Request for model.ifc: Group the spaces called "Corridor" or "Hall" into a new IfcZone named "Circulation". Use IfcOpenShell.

First a look at what the model holds.

```python
import ifcopenshell

model = ifcopenshell.open("model.ifc")
print(model.schema)
seen = {}
for space in model.by_type("IfcSpace"):
    seen[space.LongName] = seen.get(space.LongName, 0) + 1
for name, count in sorted(seen.items(), key=str):
    print(count, "x", name)
print("zones:", [z.Name for z in model.by_type("IfcZone")][:20])
```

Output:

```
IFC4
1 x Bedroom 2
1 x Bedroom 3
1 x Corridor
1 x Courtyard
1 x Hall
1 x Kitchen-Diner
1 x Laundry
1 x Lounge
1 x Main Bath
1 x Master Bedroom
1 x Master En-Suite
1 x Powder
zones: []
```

```python
import ifcopenshell
import ifcopenshell.api.group
import ifcopenshell.api.root

model = ifcopenshell.open("model.ifc")

names = {"Corridor", "Hall"}
spaces = [s for s in model.by_type("IfcSpace") if s.LongName in names]

zone = ifcopenshell.api.root.create_entity(model, ifc_class="IfcZone", name="Circulation")
ifcopenshell.api.group.assign_group(model, products=spaces, group=zone)
print(len(spaces), "spaces in", zone.Name)

model.write("model_rev.ifc")
```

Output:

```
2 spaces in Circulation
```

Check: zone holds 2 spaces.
